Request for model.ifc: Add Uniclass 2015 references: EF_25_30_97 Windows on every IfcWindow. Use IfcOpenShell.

First a look at what the model holds.

```python
import ifcopenshell

model = ifcopenshell.open("model.ifc")
print(model.schema)
print("classifications:", [c.Name for c in model.by_type("IfcClassification")])
for ifc_class in ("IfcDoor", "IfcRoof", "IfcStair", "IfcWall", "IfcWindow"):
    print(ifc_class, len(model.by_type(ifc_class)))
```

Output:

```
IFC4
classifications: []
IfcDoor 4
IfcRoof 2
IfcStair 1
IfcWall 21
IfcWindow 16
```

```python
import ifcopenshell
import ifcopenshell.api.classification

model = ifcopenshell.open("model.ifc")

system = ifcopenshell.api.classification.add_classification(model, classification="Uniclass 2015")

codes = {
    "IfcWindow": ("EF_25_30_97", "Windows"),
}
for ifc_class, (code, name) in codes.items():
    products = model.by_type(ifc_class)
    ifcopenshell.api.classification.add_reference(
        model, products=products, classification=system, identification=code, name=name
    )
    print(code, len(products))

model.write("model-out.ifc")
```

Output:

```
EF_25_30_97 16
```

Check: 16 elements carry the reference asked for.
